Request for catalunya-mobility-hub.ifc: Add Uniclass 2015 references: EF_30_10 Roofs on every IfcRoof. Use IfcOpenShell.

First a look at what the model holds.

```python
import ifcopenshell

model = ifcopenshell.open("catalunya-mobility-hub.ifc")
print(model.schema)
print("classifications:", [c.Name for c in model.by_type("IfcClassification")])
for ifc_class in ("IfcDoor", "IfcRoof", "IfcStair", "IfcWall", "IfcWindow"):
    print(ifc_class, len(model.by_type(ifc_class)))
```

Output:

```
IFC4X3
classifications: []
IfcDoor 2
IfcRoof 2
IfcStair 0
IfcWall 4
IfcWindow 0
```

```python
import ifcopenshell
import ifcopenshell.api.classification

model = ifcopenshell.open("catalunya-mobility-hub.ifc")

system = ifcopenshell.api.classification.add_classification(model, classification="Uniclass 2015")

codes = {
    "IfcRoof": ("EF_30_10", "Roofs"),
}
for ifc_class, (code, name) in codes.items():
    products = model.by_type(ifc_class)
    ifcopenshell.api.classification.add_reference(
        model, products=products, classification=system, identification=code, name=name
    )
    print(code, len(products))

model.write("catalunya-mobility-hub_edited.ifc")
```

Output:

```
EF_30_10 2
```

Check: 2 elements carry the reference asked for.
